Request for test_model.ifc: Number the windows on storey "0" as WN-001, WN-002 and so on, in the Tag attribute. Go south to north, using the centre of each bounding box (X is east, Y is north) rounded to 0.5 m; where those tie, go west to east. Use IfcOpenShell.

First a look at what the model holds.

```python
import ifcopenshell
import ifcopenshell.util.element
import ifcopenshell.util.placement

model = ifcopenshell.open("test_model.ifc")
print(model.schema)
storey = next(s for s in model.by_type("IfcBuildingStorey") if s.Name == "0")
windows = [e for e in ifcopenshell.util.element.get_decomposition(storey) if e.is_a("IfcWindow")]
for e in sorted(windows, key=lambda e: e.id()):
    origin = ifcopenshell.util.placement.get_local_placement(e.ObjectPlacement)[:3, 3]
    print(e.id(), e.Tag, e.Name, origin.round(2) + 0.0, sep=" | ")
```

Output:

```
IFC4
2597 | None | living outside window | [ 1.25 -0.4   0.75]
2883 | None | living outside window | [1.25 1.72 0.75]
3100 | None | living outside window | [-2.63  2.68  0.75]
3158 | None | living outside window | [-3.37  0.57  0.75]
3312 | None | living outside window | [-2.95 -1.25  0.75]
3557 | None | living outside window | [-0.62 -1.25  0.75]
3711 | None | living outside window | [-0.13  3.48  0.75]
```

```python
import ifcopenshell
import ifcopenshell.geom
import ifcopenshell.util.element
import ifcopenshell.util.shape

model = ifcopenshell.open("test_model.ifc")
settings = ifcopenshell.geom.settings()
settings.set("use-world-coords", True)


def centre(element):
    shape = ifcopenshell.geom.create_shape(settings, element)
    return ifcopenshell.util.shape.get_bbox_centroid(shape.geometry)


storey = next(s for s in model.by_type("IfcBuildingStorey") if s.Name == "0")
windows = [e for e in ifcopenshell.util.element.get_decomposition(storey) if e.is_a("IfcWindow")]

# Insertion points can sit at a corner or the storey origin, so sort by the geometry (in metres).
centres = {e: centre(e) for e in windows}
windows.sort(key=lambda e: (round(centres[e][1] / 0.5), centres[e][0]))

for i, e in enumerate(windows, start=1):
    number = f"WN-0{i:02d}"
    e.Tag = number
    print(e.id(), number)

model.write("test_model_v2.ifc")
```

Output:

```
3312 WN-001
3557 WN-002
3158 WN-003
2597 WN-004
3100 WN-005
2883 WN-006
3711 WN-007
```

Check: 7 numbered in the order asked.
